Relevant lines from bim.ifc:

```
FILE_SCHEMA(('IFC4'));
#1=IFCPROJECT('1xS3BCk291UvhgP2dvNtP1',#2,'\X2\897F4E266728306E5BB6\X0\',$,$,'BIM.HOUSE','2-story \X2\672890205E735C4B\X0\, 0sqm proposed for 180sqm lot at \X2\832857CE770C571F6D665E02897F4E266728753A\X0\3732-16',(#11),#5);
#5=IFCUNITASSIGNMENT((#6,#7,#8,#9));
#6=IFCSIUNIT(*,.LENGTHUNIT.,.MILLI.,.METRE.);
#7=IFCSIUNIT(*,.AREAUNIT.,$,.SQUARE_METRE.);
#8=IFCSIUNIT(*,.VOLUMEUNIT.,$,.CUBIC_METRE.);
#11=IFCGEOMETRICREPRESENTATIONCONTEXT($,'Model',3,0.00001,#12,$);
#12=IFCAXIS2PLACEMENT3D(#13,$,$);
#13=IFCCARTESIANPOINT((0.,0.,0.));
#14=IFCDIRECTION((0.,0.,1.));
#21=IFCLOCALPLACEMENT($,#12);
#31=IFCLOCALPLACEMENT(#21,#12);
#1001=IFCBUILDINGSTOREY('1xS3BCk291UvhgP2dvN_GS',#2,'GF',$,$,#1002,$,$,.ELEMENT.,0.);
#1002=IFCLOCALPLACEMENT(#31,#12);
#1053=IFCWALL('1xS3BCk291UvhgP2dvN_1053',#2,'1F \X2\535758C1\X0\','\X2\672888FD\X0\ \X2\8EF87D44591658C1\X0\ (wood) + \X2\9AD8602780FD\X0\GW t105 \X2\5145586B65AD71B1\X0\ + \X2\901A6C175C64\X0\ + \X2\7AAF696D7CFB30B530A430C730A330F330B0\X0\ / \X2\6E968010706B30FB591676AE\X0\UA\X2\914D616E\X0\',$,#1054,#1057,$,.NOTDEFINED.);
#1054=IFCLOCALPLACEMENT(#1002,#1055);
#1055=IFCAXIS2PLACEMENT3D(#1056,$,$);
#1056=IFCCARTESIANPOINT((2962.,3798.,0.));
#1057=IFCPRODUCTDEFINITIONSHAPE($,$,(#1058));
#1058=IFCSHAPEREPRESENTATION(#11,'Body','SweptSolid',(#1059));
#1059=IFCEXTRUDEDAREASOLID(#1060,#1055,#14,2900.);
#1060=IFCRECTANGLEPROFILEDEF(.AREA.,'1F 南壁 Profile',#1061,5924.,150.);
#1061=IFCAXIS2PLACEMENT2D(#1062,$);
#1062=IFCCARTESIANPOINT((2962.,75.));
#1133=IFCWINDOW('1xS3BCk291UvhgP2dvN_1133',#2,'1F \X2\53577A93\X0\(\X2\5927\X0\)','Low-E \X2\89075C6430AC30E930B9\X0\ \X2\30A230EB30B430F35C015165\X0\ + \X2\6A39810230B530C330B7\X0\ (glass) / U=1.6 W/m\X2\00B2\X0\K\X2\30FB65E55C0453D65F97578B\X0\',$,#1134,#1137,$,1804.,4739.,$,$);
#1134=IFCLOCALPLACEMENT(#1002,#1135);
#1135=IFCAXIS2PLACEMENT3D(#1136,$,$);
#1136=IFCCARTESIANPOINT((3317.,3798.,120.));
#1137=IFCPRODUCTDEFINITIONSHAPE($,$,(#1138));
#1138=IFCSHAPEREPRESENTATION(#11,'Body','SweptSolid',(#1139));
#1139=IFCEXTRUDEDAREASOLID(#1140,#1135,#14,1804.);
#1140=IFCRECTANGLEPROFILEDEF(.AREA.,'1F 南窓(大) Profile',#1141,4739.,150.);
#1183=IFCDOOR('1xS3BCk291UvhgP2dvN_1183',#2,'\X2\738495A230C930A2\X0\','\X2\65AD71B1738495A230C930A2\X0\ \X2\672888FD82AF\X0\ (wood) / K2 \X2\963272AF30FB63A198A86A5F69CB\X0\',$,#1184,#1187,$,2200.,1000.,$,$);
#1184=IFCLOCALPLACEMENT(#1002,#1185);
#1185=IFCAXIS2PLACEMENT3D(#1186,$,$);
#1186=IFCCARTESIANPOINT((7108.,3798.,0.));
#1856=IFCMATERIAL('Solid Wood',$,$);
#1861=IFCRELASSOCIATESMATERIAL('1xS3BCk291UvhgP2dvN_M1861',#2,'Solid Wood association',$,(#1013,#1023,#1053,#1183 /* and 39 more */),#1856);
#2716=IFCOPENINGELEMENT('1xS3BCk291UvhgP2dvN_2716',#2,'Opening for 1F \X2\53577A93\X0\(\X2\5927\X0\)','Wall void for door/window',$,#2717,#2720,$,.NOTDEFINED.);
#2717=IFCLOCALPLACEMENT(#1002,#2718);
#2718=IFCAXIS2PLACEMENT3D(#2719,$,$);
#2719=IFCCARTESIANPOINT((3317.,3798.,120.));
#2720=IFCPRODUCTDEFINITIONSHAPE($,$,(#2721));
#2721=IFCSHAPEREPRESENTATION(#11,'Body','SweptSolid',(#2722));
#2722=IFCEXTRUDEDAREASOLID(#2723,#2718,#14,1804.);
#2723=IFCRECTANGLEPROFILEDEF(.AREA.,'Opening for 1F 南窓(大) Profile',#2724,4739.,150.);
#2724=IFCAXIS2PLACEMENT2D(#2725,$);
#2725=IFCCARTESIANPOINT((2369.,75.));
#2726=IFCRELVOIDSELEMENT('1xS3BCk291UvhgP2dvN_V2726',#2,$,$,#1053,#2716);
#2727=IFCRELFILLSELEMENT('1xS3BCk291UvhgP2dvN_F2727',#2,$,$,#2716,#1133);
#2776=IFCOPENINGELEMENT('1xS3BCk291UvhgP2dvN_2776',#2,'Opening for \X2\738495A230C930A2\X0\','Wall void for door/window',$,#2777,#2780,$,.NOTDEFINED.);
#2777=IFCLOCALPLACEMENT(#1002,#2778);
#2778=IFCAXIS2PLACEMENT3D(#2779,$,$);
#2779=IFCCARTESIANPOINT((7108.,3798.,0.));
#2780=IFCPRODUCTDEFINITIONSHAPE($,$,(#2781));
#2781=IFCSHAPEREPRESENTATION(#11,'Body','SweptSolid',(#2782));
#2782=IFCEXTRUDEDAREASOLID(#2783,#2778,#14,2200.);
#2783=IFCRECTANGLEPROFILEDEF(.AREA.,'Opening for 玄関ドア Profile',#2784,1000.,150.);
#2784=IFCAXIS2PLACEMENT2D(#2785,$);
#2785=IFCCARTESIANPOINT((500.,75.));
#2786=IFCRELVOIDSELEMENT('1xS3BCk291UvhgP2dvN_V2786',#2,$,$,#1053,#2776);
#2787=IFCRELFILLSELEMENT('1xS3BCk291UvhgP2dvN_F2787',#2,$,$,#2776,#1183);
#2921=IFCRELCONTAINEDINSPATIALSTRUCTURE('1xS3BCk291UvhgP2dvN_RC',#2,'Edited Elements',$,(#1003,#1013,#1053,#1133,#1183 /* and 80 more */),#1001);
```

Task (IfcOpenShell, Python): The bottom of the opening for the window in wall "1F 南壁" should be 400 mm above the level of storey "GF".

```python
import numpy as np
import ifcopenshell
import ifcopenshell.api.geometry
import ifcopenshell.geom
import ifcopenshell.util.element
import ifcopenshell.util.placement
import ifcopenshell.util.shape
import ifcopenshell.util.unit

model = ifcopenshell.open("bim.ifc")
unit_scale = ifcopenshell.util.unit.calculate_unit_scale(model)

window = model.by_id(1133)
opening = window.FillsVoids[0].RelatingOpeningElement
storey = ifcopenshell.util.element.get_container(window, ifc_class="IfcBuildingStorey")
level = ifcopenshell.util.placement.get_local_placement(storey.ObjectPlacement)[2, 3]

# The opening's origin need not be at the sill, so measure its lowest point.
shape = ifcopenshell.geom.create_shape(ifcopenshell.geom.settings(), opening)
bottom = ifcopenshell.util.shape.get_shape_bottom_elevation(shape, shape.geometry) / unit_scale
dz = level + 0.4 / unit_scale - bottom

shift = np.array([0.0, 0.0, dz])
# The window is not placed relative to its opening, so move both.
for product in (opening, window):
    matrix = ifcopenshell.util.placement.get_local_placement(product.ObjectPlacement)
    matrix[:3, 3] += shift
    ifcopenshell.api.geometry.edit_object_placement(model, product=product, matrix=matrix, is_si=False)

print(f"moved by {dz * unit_scale:+.3f} m")

model.write("bim_rev.ifc")
```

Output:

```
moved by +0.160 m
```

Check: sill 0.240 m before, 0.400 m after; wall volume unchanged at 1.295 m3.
